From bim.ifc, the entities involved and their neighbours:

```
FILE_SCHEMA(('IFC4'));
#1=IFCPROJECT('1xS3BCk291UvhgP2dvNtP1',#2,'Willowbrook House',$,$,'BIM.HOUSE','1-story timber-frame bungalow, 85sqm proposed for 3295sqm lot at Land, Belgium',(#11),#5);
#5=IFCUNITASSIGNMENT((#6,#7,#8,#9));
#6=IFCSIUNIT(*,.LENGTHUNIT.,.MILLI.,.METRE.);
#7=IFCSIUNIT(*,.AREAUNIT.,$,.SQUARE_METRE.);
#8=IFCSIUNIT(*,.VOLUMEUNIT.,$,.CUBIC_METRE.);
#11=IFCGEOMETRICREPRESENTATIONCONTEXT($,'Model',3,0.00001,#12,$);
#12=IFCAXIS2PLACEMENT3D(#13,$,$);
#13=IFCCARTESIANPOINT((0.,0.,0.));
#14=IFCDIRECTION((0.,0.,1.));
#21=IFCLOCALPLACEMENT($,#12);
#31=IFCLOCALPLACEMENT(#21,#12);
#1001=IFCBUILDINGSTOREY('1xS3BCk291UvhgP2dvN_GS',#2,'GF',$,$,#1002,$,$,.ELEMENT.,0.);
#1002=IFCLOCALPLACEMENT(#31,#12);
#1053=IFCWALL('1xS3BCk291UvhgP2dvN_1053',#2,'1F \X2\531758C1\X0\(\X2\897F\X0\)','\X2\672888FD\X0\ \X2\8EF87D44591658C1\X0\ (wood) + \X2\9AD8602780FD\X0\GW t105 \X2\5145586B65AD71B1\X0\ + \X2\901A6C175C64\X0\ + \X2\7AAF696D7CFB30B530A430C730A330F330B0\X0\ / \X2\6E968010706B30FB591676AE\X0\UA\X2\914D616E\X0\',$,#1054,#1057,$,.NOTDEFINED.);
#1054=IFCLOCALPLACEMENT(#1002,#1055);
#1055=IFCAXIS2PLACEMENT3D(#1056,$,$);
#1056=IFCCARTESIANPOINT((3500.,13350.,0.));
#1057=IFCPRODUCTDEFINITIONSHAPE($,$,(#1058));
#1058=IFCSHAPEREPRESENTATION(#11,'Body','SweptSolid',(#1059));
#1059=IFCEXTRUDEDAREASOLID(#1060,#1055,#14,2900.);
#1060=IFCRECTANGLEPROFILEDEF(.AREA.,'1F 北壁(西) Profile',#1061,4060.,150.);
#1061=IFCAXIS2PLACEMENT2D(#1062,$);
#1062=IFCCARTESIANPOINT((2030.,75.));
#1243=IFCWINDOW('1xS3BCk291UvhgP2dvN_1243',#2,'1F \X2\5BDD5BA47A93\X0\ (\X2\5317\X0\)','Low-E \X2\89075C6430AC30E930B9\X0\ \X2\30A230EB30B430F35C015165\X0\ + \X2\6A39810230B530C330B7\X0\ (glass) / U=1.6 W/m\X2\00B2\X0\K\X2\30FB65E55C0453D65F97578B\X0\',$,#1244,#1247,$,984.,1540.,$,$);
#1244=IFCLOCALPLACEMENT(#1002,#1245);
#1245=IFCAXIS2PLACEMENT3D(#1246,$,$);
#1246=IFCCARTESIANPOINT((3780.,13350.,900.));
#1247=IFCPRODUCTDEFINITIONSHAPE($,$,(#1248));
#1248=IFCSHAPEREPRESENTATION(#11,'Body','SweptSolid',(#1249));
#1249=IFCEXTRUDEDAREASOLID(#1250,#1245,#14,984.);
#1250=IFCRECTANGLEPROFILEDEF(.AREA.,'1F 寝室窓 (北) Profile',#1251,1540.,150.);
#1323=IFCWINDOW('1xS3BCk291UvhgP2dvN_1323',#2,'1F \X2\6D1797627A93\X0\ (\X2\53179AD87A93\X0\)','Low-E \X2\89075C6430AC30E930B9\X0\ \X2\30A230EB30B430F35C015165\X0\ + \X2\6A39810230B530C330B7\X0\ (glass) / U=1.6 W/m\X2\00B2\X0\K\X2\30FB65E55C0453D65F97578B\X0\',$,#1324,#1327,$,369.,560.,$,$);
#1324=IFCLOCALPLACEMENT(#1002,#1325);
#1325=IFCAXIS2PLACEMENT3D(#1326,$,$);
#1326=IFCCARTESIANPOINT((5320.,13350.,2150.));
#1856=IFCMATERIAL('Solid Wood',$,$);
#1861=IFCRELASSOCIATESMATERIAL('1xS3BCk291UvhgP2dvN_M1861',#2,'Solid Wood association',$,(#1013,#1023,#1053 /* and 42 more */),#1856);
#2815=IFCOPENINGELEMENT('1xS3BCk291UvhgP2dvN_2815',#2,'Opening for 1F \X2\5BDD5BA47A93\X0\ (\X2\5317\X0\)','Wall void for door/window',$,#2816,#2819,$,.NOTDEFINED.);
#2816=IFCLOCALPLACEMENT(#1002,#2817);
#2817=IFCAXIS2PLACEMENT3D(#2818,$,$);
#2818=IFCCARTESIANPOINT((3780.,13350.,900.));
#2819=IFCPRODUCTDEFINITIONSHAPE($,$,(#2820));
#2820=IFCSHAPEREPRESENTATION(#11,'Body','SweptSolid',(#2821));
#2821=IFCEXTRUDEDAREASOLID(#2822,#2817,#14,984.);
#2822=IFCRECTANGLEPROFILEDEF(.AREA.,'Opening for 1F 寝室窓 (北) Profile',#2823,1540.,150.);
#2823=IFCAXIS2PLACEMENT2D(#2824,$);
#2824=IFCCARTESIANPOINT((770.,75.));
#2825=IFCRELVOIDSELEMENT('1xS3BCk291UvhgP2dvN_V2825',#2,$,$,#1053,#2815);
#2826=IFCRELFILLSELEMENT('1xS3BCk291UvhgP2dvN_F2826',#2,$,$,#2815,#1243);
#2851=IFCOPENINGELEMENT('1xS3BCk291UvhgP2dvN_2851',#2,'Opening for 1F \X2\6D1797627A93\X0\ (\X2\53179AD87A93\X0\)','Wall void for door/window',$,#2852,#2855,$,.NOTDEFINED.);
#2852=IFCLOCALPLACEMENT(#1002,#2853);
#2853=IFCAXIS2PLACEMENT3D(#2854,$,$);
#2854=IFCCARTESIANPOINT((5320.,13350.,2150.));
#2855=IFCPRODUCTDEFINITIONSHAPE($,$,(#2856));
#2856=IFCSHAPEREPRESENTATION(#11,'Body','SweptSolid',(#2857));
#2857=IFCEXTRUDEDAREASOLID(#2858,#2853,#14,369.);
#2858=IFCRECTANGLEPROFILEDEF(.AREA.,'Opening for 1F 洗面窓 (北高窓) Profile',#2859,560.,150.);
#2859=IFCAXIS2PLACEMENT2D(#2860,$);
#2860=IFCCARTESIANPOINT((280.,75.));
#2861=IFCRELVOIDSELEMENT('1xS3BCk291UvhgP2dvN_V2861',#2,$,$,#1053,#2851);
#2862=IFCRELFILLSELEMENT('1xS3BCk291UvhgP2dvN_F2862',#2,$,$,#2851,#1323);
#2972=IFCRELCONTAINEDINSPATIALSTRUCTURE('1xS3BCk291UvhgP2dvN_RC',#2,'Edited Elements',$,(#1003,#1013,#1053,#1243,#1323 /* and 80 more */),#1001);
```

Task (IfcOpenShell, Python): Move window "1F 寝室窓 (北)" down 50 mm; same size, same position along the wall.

```python
import numpy as np
import ifcopenshell
import ifcopenshell.api.geometry
import ifcopenshell.util.placement
import ifcopenshell.util.unit

model = ifcopenshell.open("bim.ifc")
unit_scale = ifcopenshell.util.unit.calculate_unit_scale(model)

window = model.by_guid("1xS3BCk291UvhgP2dvN_1243")
opening = window.FillsVoids[0].RelatingOpeningElement
dz = -50.0

shift = np.array([0.0, 0.0, dz])
# The window is not placed relative to its opening, so move both.
for product in (opening, window):
    matrix = ifcopenshell.util.placement.get_local_placement(product.ObjectPlacement)
    matrix[:3, 3] += shift
    ifcopenshell.api.geometry.edit_object_placement(model, product=product, matrix=matrix, is_si=False)

print(f"moved by {dz * unit_scale:+.3f} m")

model.write("bim_updated.ifc")
```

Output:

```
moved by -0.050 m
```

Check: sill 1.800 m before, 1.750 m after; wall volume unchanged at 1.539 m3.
